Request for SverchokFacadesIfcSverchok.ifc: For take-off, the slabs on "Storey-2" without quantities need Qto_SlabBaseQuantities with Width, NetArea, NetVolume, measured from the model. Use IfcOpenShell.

First a look at what the model holds.

```python
import ifcopenshell
import ifcopenshell.util.element
import ifcopenshell.util.unit

model = ifcopenshell.open("SverchokFacadesIfcSverchok.ifc")
print(model.schema)
for unit_type in ("LENGTHUNIT", "AREAUNIT", "VOLUMEUNIT"):
    print(unit_type, ifcopenshell.util.unit.calculate_unit_scale(model, unit_type))
storey = next(s for s in model.by_type("IfcBuildingStorey") if s.Name == "Storey-2")
slabs = [e for e in ifcopenshell.util.element.get_decomposition(storey) if e.is_a("IfcSlab")]
for e in sorted(slabs, key=lambda e: e.id()):
    print(e.id(), e.is_a(), e.Name, list(ifcopenshell.util.element.get_psets(e, qtos_only=True)), sep=" | ")
```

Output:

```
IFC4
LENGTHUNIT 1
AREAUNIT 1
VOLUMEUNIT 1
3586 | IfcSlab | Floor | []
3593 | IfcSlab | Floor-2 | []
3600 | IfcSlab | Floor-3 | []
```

```python
import ifcopenshell
import ifcopenshell.api.pset
import ifcopenshell.geom
import ifcopenshell.util.element
import ifcopenshell.util.shape
import ifcopenshell.util.unit

model = ifcopenshell.open("SverchokFacadesIfcSverchok.ifc")
unit_scale = ifcopenshell.util.unit.calculate_unit_scale(model)
area_scale = ifcopenshell.util.unit.calculate_unit_scale(model, "AREAUNIT")
volume_scale = ifcopenshell.util.unit.calculate_unit_scale(model, "VOLUMEUNIT")
settings = ifcopenshell.geom.settings()

storey = next(s for s in model.by_type("IfcBuildingStorey") if s.Name == "Storey-2")
slabs = [e for e in ifcopenshell.util.element.get_decomposition(storey) if e.is_a("IfcSlab")]

for e in sorted(slabs, key=lambda e: e.id()):
    if ifcopenshell.util.element.get_psets(e, qtos_only=True, should_inherit=False):
        continue
    # Geometry comes back in metres, in the element's own axes.
    shape = ifcopenshell.geom.create_shape(settings, e)
    values = {
        "Width": ifcopenshell.util.shape.get_z(shape.geometry) / unit_scale,
        "NetArea": ifcopenshell.util.shape.get_footprint_area(shape.geometry) / area_scale,
        "NetVolume": ifcopenshell.util.shape.get_volume(shape.geometry) / volume_scale,
    }
    qto = ifcopenshell.api.pset.add_qto(model, product=e, name="Qto_SlabBaseQuantities")
    ifcopenshell.api.pset.edit_qto(model, qto=qto, properties=values)
    print(e.id(), {k: round(v, 3) for k, v in values.items()})

model.write("SverchokFacadesIfcSverchok_updated.ifc")
```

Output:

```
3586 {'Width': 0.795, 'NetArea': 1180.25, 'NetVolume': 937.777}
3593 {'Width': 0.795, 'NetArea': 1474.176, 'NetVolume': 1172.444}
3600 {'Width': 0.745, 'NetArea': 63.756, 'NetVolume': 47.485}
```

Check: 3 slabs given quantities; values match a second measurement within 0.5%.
